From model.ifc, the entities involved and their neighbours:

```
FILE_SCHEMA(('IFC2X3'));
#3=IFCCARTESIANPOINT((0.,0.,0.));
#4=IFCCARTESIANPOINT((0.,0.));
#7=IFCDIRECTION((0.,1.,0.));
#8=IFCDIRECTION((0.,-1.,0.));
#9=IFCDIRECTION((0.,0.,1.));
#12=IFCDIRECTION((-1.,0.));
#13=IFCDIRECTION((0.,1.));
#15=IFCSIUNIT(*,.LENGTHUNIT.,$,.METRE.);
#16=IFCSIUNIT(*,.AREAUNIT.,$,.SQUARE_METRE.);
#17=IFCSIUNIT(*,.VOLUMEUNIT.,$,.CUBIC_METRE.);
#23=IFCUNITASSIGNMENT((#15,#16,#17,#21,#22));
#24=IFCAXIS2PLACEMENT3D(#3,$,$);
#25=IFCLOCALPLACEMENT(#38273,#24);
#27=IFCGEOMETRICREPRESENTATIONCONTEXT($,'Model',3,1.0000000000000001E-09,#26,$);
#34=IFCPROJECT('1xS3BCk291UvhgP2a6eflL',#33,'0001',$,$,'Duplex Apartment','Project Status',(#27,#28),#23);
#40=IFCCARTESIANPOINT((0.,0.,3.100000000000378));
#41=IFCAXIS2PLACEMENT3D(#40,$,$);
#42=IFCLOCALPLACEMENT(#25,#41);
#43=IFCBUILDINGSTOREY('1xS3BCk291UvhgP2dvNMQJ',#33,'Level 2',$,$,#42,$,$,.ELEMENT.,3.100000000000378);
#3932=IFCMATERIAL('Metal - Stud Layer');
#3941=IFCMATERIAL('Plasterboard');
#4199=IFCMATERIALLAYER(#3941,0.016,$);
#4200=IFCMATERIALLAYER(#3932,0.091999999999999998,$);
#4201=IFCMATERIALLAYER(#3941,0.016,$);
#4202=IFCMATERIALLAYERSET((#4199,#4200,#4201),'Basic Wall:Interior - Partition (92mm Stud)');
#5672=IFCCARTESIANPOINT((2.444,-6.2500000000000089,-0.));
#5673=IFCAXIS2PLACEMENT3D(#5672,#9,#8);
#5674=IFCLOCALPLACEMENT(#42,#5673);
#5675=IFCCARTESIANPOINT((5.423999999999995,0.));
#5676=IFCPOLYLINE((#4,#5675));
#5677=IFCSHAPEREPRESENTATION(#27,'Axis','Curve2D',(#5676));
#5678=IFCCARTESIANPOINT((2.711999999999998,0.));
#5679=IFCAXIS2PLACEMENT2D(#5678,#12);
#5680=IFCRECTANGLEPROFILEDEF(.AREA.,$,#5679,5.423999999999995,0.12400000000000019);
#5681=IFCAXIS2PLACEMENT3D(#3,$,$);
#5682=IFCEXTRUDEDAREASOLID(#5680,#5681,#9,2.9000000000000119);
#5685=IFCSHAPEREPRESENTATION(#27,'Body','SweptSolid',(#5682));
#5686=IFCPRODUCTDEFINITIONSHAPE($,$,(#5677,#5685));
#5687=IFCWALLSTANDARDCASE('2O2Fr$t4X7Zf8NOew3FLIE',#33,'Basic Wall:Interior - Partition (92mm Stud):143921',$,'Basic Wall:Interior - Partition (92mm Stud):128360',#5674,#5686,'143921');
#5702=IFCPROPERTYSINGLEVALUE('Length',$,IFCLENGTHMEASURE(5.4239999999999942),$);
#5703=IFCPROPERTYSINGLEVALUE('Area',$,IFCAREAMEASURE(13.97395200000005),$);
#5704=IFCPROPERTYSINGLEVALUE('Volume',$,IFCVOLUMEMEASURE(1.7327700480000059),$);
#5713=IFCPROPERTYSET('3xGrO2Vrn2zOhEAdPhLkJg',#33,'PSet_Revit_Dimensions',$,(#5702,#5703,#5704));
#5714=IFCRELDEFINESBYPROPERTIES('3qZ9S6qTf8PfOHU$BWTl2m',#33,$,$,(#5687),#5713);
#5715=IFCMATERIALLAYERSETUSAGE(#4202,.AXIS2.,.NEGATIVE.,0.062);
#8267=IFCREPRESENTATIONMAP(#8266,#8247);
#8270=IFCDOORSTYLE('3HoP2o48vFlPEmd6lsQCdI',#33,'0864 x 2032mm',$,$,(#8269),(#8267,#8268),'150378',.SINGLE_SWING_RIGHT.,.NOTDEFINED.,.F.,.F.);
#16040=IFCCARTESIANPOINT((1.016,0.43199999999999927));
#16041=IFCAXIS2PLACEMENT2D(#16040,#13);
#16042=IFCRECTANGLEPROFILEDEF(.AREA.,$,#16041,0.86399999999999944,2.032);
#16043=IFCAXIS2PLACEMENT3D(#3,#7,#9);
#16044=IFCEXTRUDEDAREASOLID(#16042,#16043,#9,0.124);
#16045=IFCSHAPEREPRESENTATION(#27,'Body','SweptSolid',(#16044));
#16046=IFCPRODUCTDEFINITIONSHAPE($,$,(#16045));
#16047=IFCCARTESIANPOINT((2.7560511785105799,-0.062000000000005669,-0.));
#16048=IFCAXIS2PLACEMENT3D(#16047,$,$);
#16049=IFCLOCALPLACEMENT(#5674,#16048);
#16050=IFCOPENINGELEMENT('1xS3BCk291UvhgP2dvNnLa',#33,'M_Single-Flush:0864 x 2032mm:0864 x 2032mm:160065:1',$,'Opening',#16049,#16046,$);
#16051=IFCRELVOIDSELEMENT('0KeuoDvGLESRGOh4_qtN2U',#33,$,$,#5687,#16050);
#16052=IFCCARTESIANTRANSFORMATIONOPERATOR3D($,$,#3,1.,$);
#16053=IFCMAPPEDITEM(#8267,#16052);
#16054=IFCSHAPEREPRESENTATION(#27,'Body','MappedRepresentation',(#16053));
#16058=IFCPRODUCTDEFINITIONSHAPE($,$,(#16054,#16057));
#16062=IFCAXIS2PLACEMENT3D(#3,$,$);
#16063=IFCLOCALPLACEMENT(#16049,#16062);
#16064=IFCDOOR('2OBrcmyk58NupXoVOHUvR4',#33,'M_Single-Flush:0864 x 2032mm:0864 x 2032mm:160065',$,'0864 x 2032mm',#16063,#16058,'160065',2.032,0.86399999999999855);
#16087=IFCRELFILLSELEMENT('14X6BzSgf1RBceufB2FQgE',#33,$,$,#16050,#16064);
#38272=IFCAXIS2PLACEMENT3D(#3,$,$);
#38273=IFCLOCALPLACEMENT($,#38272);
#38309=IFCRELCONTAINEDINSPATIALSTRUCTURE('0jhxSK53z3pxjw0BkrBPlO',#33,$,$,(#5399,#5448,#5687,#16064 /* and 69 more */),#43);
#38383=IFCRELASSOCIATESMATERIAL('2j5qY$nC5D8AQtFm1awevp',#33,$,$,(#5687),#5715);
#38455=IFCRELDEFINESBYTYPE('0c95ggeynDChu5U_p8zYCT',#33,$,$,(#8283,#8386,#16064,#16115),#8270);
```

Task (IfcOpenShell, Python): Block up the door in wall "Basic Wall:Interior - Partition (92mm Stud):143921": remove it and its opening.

```python
import ifcopenshell
import ifcopenshell.api.feature
import ifcopenshell.api.pset
import ifcopenshell.api.root
import ifcopenshell.geom
import ifcopenshell.util.element
import ifcopenshell.util.shape
import ifcopenshell.util.unit

model = ifcopenshell.open("model.ifc")
area_scale = ifcopenshell.util.unit.calculate_unit_scale(model, "AREAUNIT")
volume_scale = ifcopenshell.util.unit.calculate_unit_scale(model, "VOLUMEUNIT")
settings = ifcopenshell.geom.settings()


def volume(element):
    """Net volume in cubic metres, openings subtracted."""
    shape = ifcopenshell.geom.create_shape(settings, element)
    return ifcopenshell.util.shape.get_volume(shape.geometry)


door = model.by_id(16064)
opening = door.FillsVoids[0].RelatingOpeningElement
wall = opening.VoidsElements[0].RelatingBuildingElement
before = volume(wall)

ifcopenshell.api.root.remove_product(model, product=door)
ifcopenshell.api.feature.remove_feature(model, feature=opening)

after = volume(wall)
thickness = 0.124  # wall thickness in metres

# Update the wall's stored quantities.
pset = model.by_id(ifcopenshell.util.element.get_pset(wall, "PSet_Revit_Dimensions", should_inherit=False)["id"])
ifcopenshell.api.pset.edit_pset(model, pset=pset, properties={
    "Area": model.create_entity("IfcAreaMeasure", after / thickness / area_scale),
    "Volume": model.create_entity("IfcVolumeMeasure", after / volume_scale),
})

print(f"wall volume {before:.3f} -> {after:.3f} m3")

model.write("model_rev.ifc")
```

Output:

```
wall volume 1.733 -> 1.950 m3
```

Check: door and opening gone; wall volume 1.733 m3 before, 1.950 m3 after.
